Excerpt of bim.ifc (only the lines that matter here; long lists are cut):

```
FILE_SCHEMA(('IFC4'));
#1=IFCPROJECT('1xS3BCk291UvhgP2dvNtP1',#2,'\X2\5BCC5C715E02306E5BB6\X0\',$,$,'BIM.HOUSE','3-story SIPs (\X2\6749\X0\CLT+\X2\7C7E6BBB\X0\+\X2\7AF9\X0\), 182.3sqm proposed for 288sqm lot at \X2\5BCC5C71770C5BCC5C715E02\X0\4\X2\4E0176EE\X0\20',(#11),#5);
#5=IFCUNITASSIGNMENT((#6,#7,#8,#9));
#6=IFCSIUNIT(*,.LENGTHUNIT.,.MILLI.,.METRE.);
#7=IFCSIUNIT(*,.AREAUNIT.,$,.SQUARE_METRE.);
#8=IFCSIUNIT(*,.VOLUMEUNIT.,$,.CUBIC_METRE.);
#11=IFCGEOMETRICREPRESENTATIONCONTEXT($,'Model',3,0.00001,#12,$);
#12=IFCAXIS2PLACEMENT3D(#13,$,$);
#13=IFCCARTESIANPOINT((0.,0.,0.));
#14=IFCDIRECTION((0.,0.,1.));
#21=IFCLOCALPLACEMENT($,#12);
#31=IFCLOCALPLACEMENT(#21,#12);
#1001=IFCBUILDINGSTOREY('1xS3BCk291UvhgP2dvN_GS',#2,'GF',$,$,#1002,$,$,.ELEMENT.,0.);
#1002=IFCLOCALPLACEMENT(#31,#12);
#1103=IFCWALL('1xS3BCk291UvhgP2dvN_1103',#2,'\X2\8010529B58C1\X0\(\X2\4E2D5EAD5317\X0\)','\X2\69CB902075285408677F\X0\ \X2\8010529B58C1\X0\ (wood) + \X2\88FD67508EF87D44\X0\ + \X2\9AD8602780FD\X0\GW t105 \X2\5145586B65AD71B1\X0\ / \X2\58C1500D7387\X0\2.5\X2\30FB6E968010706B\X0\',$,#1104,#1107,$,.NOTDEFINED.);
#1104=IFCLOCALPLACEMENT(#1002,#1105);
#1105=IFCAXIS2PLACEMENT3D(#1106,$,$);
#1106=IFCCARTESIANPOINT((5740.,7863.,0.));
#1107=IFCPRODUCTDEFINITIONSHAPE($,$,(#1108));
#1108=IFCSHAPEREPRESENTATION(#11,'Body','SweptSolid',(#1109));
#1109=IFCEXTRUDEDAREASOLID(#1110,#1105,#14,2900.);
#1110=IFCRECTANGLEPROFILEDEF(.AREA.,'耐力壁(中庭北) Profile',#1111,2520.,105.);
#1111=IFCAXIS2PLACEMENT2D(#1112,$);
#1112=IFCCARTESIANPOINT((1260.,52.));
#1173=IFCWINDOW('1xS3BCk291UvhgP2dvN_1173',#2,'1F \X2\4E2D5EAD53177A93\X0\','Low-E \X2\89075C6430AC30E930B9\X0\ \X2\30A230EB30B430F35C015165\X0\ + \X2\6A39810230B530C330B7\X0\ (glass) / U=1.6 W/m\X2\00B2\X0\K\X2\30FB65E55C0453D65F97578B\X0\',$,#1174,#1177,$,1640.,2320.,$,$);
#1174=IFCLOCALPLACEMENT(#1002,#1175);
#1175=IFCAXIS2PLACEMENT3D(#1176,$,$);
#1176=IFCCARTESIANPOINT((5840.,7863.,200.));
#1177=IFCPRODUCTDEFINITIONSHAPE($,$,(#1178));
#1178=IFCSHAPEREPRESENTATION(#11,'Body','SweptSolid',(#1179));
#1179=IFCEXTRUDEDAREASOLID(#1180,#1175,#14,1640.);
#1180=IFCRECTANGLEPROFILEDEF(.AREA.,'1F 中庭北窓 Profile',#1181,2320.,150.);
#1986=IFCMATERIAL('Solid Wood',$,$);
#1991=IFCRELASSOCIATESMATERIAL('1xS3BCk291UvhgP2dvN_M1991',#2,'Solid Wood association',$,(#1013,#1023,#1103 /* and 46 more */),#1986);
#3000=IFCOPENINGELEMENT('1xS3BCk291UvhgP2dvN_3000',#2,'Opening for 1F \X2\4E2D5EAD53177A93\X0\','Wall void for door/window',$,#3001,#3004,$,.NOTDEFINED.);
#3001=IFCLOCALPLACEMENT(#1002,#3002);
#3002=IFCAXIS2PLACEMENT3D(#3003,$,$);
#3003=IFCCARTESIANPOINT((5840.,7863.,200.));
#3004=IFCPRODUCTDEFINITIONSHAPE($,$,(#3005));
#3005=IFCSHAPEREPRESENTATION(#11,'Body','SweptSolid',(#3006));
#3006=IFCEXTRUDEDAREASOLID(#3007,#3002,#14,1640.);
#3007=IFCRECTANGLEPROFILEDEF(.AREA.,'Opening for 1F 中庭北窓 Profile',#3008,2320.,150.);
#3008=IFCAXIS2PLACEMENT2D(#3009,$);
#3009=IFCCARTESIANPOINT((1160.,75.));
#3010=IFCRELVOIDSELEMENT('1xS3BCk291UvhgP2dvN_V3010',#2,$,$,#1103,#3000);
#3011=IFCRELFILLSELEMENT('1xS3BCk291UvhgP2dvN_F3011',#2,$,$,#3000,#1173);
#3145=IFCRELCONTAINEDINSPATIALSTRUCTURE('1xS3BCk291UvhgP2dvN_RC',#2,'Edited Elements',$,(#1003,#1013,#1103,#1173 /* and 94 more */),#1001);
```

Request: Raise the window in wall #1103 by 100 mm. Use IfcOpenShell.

```python
import numpy as np
import ifcopenshell
import ifcopenshell.api.geometry
import ifcopenshell.util.placement
import ifcopenshell.util.unit

model = ifcopenshell.open("bim.ifc")
unit_scale = ifcopenshell.util.unit.calculate_unit_scale(model)

window = model.by_id(1173)
opening = window.FillsVoids[0].RelatingOpeningElement
dz = 100.0

shift = np.array([0.0, 0.0, dz])
# The window is not placed relative to its opening, so move both.
for product in (opening, window):
    matrix = ifcopenshell.util.placement.get_local_placement(product.ObjectPlacement)
    matrix[:3, 3] += shift
    ifcopenshell.api.geometry.edit_object_placement(model, product=product, matrix=matrix, is_si=False)

print(f"moved by {dz * unit_scale:+.3f} m")

model.write("bim-out.ifc")
```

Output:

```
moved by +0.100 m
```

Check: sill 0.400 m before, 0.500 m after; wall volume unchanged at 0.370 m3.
